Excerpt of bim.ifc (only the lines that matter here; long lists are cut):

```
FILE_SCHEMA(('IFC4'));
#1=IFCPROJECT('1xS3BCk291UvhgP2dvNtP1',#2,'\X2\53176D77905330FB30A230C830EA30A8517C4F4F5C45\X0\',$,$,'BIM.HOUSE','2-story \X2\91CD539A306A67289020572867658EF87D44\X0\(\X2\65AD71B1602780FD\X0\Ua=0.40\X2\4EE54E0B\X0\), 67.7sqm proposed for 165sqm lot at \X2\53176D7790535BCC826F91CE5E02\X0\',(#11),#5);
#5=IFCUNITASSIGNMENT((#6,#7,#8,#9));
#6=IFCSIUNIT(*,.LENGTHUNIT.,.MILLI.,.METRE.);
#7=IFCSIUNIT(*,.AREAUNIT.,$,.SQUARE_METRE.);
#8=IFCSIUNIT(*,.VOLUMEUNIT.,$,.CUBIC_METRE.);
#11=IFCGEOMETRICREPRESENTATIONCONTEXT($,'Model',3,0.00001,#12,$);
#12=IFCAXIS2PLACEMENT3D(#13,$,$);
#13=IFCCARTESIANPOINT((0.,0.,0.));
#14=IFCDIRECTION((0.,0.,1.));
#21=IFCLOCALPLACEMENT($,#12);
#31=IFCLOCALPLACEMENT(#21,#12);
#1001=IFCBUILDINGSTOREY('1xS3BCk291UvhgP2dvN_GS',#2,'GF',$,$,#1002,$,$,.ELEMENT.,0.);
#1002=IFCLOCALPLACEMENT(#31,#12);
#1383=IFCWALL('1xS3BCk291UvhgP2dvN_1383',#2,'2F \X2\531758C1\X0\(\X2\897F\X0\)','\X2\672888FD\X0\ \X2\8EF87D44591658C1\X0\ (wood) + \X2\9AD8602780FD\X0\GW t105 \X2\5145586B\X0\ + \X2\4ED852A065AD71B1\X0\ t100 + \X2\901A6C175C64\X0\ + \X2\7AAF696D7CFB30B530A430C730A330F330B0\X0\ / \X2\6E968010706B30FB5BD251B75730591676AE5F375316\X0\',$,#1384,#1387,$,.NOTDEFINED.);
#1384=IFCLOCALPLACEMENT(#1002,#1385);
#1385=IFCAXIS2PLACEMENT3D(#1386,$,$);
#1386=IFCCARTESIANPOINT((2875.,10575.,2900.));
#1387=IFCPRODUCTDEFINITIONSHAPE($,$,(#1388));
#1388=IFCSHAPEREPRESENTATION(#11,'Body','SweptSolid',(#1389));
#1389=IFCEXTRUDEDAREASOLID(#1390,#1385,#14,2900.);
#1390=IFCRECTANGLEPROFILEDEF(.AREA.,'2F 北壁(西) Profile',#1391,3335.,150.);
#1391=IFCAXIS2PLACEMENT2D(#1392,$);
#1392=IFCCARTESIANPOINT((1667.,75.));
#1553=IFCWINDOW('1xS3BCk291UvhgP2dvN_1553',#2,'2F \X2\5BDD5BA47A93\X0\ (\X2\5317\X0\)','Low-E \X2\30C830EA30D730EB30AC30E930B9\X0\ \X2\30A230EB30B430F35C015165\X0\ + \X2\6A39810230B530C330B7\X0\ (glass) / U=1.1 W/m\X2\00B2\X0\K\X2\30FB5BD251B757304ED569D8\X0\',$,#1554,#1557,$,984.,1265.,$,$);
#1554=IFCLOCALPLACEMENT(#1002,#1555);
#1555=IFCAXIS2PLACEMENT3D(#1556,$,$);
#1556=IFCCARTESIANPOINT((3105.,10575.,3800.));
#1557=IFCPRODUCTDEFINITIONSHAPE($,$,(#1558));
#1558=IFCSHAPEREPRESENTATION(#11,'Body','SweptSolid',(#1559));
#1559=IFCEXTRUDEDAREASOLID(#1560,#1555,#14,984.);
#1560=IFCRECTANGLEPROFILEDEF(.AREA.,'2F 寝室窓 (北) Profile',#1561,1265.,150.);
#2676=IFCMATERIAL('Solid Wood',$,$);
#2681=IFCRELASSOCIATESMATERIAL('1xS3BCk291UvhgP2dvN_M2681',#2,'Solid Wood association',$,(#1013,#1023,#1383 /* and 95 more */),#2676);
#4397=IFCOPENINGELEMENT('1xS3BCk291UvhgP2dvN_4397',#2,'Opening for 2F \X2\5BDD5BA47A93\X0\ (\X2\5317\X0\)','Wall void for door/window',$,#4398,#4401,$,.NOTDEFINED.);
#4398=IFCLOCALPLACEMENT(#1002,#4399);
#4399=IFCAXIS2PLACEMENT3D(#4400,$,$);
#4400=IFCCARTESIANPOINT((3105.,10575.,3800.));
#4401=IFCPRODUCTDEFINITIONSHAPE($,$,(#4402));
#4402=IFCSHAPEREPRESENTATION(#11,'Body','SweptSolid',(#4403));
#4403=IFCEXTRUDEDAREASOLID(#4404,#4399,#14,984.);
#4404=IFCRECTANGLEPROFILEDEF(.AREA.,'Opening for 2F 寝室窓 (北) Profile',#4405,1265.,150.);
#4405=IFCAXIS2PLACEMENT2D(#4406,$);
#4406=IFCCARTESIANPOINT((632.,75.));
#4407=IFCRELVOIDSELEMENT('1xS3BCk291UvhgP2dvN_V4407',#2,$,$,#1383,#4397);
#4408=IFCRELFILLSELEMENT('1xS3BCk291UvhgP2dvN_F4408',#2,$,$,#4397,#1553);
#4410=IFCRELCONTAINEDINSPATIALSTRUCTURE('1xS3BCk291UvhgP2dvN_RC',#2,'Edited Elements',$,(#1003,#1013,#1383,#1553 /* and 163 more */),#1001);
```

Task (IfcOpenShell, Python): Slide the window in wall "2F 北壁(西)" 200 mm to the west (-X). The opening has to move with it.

```python
import ifcopenshell
import ifcopenshell.api.geometry
import ifcopenshell.util.placement

model = ifcopenshell.open("bim.ifc")

window = model.by_id(1553)
opening = window.FillsVoids[0].RelatingOpeningElement
wall = opening.VoidsElements[0].RelatingBuildingElement

wall_matrix = ifcopenshell.util.placement.get_local_placement(wall.ObjectPlacement)
shift = wall_matrix[:3, 0] * -200.0
before = ifcopenshell.util.placement.get_local_placement(window.ObjectPlacement)[:3, 3].copy()

# The window is not placed relative to its opening, so move both.
for product in (opening, window):
    matrix = ifcopenshell.util.placement.get_local_placement(product.ObjectPlacement)
    matrix[:3, 3] += shift
    ifcopenshell.api.geometry.edit_object_placement(model, product=product, matrix=matrix, is_si=False)

after = ifcopenshell.util.placement.get_local_placement(window.ObjectPlacement)[:3, 3]
print("window moved by", (after - before).round(3) + 0.0)

model.write("bim-out.ifc")
```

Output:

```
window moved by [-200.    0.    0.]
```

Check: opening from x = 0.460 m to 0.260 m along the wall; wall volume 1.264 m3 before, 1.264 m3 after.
